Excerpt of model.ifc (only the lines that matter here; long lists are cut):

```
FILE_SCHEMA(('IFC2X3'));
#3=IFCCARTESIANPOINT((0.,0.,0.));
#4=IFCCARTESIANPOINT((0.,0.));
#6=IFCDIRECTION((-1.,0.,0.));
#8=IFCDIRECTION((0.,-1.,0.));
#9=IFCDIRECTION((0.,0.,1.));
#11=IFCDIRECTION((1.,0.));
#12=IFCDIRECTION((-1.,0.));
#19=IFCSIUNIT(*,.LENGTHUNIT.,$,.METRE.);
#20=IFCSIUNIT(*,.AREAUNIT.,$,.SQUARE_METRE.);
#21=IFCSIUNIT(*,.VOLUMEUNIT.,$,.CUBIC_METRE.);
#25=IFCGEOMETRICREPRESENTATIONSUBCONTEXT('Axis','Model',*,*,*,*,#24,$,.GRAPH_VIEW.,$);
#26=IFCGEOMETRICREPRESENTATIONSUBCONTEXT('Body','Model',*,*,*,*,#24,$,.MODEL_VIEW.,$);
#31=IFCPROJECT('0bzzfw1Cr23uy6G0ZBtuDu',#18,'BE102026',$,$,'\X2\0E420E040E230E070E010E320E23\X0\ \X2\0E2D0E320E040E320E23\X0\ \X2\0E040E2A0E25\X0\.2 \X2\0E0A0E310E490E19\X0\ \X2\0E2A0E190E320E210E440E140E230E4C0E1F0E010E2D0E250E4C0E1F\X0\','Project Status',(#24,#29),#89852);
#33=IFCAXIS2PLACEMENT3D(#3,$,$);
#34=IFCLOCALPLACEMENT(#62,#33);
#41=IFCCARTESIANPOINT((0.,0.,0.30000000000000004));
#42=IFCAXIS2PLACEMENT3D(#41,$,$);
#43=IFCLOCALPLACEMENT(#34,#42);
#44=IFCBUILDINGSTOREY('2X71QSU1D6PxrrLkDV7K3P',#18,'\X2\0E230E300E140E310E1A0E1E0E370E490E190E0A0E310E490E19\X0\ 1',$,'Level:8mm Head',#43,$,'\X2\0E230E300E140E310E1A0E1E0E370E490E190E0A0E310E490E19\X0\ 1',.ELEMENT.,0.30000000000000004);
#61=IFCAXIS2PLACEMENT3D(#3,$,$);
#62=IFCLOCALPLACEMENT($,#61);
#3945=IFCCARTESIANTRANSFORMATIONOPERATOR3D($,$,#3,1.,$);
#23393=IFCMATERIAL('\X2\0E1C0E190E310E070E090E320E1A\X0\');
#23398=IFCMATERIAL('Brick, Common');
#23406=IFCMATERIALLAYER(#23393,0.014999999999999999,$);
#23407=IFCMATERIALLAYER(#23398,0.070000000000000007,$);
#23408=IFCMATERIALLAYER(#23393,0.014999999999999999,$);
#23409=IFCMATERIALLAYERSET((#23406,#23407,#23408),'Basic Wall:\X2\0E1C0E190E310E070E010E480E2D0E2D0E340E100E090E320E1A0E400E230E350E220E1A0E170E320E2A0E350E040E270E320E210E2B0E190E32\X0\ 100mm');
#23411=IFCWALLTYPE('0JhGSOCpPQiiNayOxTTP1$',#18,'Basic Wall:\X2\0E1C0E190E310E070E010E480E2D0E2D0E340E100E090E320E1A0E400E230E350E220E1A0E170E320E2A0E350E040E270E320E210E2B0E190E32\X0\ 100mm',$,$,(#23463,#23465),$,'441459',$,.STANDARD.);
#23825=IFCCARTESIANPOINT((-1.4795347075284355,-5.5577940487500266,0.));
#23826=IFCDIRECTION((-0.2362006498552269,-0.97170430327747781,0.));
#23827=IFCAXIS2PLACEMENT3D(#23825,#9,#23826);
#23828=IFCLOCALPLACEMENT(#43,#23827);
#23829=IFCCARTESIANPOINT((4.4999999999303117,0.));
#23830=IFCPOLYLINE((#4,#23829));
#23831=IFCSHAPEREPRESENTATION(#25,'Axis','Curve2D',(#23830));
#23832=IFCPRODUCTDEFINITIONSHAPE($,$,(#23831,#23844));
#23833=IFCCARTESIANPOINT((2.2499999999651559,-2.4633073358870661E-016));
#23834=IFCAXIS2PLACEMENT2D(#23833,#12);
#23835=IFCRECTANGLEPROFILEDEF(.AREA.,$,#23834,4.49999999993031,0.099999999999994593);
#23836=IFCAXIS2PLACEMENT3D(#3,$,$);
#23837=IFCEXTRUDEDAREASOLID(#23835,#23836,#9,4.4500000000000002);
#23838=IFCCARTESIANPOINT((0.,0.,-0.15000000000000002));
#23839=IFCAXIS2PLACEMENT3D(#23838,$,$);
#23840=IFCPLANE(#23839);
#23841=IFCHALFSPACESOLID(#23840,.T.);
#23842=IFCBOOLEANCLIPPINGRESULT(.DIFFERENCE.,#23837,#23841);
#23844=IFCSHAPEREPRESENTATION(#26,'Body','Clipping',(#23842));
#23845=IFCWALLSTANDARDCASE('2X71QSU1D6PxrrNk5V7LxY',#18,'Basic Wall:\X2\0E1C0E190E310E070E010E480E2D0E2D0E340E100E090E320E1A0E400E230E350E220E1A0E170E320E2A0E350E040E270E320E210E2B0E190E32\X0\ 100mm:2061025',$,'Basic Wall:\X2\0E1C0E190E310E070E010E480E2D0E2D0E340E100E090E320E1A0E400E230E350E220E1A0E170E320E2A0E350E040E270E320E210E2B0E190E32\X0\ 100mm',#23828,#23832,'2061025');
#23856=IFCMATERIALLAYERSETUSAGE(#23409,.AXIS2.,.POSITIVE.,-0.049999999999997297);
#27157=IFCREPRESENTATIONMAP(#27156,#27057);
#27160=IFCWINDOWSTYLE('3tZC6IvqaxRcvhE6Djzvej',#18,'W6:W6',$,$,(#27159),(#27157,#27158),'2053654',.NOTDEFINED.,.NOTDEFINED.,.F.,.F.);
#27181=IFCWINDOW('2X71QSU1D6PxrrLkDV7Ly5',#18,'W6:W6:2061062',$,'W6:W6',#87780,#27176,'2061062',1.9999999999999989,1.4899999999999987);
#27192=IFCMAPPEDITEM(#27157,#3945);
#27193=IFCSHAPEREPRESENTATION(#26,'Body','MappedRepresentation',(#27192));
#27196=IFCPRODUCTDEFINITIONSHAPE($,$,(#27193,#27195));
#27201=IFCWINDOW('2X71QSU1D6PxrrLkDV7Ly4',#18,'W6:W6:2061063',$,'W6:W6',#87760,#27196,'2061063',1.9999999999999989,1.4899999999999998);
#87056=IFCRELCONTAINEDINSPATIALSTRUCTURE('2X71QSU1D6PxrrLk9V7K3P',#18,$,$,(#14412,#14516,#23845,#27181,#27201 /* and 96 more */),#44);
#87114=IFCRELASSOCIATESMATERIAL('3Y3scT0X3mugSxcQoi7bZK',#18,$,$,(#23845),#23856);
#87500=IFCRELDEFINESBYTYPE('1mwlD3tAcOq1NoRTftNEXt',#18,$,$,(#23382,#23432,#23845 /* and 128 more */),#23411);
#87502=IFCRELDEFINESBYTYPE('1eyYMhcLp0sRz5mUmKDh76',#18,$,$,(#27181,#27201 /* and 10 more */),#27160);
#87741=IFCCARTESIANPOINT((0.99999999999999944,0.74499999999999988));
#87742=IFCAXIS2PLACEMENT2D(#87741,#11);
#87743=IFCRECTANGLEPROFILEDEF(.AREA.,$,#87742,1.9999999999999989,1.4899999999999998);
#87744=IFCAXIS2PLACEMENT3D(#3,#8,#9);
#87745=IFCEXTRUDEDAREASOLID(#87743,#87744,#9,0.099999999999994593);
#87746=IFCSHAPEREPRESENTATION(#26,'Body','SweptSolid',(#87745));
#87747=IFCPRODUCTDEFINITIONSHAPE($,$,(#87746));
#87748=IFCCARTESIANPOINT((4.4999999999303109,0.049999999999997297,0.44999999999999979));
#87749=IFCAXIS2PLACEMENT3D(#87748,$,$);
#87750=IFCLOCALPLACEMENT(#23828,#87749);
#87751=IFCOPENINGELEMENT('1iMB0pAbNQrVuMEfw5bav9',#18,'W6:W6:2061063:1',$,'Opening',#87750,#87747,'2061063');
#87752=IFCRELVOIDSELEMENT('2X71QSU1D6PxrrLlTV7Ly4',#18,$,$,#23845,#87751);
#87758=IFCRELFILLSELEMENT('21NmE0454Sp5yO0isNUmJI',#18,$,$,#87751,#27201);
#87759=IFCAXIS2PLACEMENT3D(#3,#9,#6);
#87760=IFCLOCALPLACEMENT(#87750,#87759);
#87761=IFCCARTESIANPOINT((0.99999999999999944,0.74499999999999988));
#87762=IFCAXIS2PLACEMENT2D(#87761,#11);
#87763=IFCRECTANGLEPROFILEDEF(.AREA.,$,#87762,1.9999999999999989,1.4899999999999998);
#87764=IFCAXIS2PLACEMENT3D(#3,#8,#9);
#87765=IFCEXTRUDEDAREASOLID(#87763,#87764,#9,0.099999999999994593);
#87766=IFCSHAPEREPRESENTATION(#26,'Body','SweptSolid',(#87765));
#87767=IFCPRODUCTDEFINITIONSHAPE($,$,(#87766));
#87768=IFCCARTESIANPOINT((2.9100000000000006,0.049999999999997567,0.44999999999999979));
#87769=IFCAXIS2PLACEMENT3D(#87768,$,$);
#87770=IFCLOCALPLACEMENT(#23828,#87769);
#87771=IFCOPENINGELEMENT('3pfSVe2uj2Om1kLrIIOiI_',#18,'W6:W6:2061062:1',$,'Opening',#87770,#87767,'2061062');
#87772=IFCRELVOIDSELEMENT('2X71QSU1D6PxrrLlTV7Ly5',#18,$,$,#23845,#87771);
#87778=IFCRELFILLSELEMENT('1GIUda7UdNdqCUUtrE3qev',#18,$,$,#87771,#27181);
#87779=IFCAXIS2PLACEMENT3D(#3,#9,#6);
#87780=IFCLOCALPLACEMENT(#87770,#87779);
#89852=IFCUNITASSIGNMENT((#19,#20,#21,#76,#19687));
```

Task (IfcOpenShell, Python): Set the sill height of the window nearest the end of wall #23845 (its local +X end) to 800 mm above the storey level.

```python
import numpy as np
import ifcopenshell
import ifcopenshell.api.geometry
import ifcopenshell.geom
import ifcopenshell.util.element
import ifcopenshell.util.placement
import ifcopenshell.util.shape
import ifcopenshell.util.unit

model = ifcopenshell.open("model.ifc")
unit_scale = ifcopenshell.util.unit.calculate_unit_scale(model)

window = model.by_guid("2X71QSU1D6PxrrLkDV7Ly4")
opening = window.FillsVoids[0].RelatingOpeningElement
storey = ifcopenshell.util.element.get_container(window, ifc_class="IfcBuildingStorey")
level = ifcopenshell.util.placement.get_local_placement(storey.ObjectPlacement)[2, 3]

# The opening's origin need not be at the sill, so measure its lowest point.
shape = ifcopenshell.geom.create_shape(ifcopenshell.geom.settings(), opening)
bottom = ifcopenshell.util.shape.get_shape_bottom_elevation(shape, shape.geometry) / unit_scale
dz = level + 0.8 / unit_scale - bottom

shift = np.array([0.0, 0.0, dz])
# The window is placed relative to its opening, so it follows when the opening moves.
matrix = ifcopenshell.util.placement.get_local_placement(opening.ObjectPlacement)
matrix[:3, 3] += shift
ifcopenshell.api.geometry.edit_object_placement(
    model, product=opening, matrix=matrix, is_si=False, should_transform_children=True
)

print(f"moved by {dz * unit_scale:+.3f} m")

model.write("model_v2.ifc")
```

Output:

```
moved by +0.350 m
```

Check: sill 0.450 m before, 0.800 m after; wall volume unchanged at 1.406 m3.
